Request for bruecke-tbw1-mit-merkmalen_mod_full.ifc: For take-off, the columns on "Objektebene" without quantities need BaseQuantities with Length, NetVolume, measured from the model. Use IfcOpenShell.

First a look at what the model holds.

```python
import ifcopenshell
import ifcopenshell.util.element
import ifcopenshell.util.unit

model = ifcopenshell.open("bruecke-tbw1-mit-merkmalen_mod_full.ifc")
print(model.schema)
for unit_type in ("LENGTHUNIT", "AREAUNIT", "VOLUMEUNIT"):
    print(unit_type, ifcopenshell.util.unit.calculate_unit_scale(model, unit_type))
storey = next(s for s in model.by_type("IfcBuildingStorey") if s.Name == "Objektebene")
columns = [e for e in ifcopenshell.util.element.get_decomposition(storey) if e.is_a("IfcColumn")]
for e in sorted(columns, key=lambda e: e.id()):
    print(e.id(), e.is_a(), e.Name, list(ifcopenshell.util.element.get_psets(e, qtos_only=True)), sep=" | ")
```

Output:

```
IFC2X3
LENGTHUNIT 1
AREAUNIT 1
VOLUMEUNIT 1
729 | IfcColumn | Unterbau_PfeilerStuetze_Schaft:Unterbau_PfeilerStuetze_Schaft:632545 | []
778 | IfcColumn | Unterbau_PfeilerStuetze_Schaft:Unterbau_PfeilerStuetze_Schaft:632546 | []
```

```python
import ifcopenshell
import ifcopenshell.api.pset
import ifcopenshell.geom
import ifcopenshell.util.element
import ifcopenshell.util.shape
import ifcopenshell.util.unit

model = ifcopenshell.open("bruecke-tbw1-mit-merkmalen_mod_full.ifc")
unit_scale = ifcopenshell.util.unit.calculate_unit_scale(model)
volume_scale = ifcopenshell.util.unit.calculate_unit_scale(model, "VOLUMEUNIT")
settings = ifcopenshell.geom.settings()

storey = next(s for s in model.by_type("IfcBuildingStorey") if s.Name == "Objektebene")
columns = [e for e in ifcopenshell.util.element.get_decomposition(storey) if e.is_a("IfcColumn")]

for e in sorted(columns, key=lambda e: e.id()):
    if ifcopenshell.util.element.get_psets(e, qtos_only=True, should_inherit=False):
        continue
    # Geometry comes back in metres, in the element's own axes.
    shape = ifcopenshell.geom.create_shape(settings, e)
    values = {
        "Length": ifcopenshell.util.shape.get_z(shape.geometry) / unit_scale,
        "NetVolume": ifcopenshell.util.shape.get_volume(shape.geometry) / volume_scale,
    }
    qto = ifcopenshell.api.pset.add_qto(model, product=e, name="BaseQuantities")
    ifcopenshell.api.pset.edit_qto(model, qto=qto, properties=values)
    print(e.id(), {k: round(v, 3) for k, v in values.items()})

model.write("bruecke-tbw1-mit-merkmalen_mod_full_rev.ifc")
```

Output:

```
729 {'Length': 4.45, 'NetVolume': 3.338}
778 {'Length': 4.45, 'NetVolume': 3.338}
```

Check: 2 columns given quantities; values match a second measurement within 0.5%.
